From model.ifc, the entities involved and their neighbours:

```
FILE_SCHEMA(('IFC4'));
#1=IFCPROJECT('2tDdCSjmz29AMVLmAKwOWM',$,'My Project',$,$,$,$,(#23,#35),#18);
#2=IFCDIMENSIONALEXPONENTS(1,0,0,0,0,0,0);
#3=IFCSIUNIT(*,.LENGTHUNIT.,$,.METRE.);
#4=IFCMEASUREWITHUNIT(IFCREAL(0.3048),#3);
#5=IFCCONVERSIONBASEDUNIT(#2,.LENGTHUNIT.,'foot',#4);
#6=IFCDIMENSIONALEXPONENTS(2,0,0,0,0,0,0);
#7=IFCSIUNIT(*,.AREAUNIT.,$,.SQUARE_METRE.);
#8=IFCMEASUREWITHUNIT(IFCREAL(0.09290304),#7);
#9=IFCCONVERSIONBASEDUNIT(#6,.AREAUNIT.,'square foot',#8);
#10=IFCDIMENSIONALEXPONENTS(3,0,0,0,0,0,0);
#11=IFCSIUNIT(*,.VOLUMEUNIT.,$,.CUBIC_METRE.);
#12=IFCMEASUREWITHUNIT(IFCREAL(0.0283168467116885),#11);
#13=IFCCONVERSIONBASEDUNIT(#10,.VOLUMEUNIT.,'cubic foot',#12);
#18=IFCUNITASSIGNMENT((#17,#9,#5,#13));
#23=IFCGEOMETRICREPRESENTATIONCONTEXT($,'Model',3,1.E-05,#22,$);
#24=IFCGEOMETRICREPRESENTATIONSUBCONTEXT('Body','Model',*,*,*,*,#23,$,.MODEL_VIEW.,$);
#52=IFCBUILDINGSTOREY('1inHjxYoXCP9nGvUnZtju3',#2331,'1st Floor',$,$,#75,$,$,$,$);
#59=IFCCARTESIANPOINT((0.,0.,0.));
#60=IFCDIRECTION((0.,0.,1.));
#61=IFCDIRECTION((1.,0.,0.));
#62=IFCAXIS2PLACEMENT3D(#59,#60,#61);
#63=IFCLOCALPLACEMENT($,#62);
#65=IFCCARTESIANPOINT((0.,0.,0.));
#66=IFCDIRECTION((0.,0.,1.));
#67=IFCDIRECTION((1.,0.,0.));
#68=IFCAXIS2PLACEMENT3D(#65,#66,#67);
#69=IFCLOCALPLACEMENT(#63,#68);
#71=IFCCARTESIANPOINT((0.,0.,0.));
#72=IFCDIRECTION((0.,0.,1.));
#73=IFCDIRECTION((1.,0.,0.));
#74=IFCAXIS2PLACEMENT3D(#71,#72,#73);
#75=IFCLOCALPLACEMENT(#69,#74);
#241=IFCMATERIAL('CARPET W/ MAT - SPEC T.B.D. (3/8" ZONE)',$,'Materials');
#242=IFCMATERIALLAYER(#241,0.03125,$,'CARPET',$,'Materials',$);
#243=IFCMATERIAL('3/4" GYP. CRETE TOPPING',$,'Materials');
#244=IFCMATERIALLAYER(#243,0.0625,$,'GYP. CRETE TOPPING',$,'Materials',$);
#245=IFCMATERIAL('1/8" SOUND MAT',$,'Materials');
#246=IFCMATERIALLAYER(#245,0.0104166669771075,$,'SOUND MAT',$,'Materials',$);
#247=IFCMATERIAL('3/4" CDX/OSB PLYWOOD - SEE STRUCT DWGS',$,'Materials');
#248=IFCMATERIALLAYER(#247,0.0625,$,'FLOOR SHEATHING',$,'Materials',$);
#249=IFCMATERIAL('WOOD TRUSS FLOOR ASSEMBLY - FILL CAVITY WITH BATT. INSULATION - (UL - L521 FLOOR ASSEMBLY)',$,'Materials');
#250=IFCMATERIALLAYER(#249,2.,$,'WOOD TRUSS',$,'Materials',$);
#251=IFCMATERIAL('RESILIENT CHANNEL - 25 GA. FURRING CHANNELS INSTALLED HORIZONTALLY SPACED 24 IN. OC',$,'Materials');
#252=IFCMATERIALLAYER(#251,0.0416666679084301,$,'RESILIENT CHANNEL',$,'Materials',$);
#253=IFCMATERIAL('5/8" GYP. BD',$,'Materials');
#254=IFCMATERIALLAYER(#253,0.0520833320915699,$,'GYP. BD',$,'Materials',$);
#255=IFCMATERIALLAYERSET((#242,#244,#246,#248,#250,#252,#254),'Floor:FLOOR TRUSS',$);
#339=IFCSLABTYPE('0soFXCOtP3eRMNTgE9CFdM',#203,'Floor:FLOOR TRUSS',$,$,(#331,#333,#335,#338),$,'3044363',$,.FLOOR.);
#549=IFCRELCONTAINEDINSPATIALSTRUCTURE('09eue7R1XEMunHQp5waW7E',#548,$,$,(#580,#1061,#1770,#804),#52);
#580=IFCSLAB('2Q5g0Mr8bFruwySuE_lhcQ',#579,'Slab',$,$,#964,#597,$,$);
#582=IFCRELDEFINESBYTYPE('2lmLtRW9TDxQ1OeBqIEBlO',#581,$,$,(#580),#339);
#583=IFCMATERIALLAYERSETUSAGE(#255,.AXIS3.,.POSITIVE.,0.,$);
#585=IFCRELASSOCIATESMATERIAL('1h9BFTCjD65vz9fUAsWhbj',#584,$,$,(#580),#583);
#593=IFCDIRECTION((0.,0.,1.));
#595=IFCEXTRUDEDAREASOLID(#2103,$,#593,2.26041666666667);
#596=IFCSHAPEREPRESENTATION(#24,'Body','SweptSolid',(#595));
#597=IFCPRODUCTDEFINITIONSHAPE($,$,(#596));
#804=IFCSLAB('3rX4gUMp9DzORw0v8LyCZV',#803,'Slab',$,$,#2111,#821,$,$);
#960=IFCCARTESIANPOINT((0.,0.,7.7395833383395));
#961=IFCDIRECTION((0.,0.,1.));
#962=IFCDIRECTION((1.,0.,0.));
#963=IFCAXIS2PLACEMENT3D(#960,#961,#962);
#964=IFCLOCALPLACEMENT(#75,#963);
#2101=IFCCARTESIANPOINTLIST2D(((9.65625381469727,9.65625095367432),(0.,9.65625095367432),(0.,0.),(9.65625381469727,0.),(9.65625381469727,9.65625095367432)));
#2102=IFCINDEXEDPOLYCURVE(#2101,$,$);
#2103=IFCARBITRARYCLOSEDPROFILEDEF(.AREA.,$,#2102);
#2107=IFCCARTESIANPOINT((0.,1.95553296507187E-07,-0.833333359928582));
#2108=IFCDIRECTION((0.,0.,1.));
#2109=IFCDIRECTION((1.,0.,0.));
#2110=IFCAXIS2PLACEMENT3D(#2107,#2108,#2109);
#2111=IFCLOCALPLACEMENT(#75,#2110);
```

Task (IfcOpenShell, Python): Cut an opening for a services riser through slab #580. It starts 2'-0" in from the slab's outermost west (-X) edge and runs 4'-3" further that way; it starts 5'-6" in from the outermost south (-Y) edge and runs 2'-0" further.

```python
import numpy as np
import ifcopenshell
import ifcopenshell.api.feature
import ifcopenshell.api.geometry
import ifcopenshell.api.root
import ifcopenshell.geom
import ifcopenshell.util.placement
import ifcopenshell.util.representation
import ifcopenshell.util.shape
import ifcopenshell.util.unit

model = ifcopenshell.open("model.ifc")
unit_scale = ifcopenshell.util.unit.calculate_unit_scale(model)
settings = ifcopenshell.geom.settings()


def volume(element):
    """Net volume in cubic metres, openings subtracted."""
    shape = ifcopenshell.geom.create_shape(settings, element)
    return ifcopenshell.util.shape.get_volume(shape.geometry)


slab = model.by_id(580)
before = volume(slab)

# Extent in the slab's own axes, in metres. The edges named are its -X and -Y sides.
slab_shape = ifcopenshell.geom.create_shape(settings, slab)
vertices = ifcopenshell.util.shape.get_vertices(slab_shape.geometry)
x_min, y_min, bottom = vertices.min(axis=0)
top = vertices[:, 2].max()

opening = ifcopenshell.api.root.create_entity(model, ifc_class="IfcOpeningElement", name="Services riser opening", predefined_type="OPENING")
context = ifcopenshell.util.representation.get_context(model, "Model", "Body", "MODEL_VIEW")
width, depth = 1.2954, 0.6096
outline = [(0.0, 0.0), (width, 0.0), (width, depth), (0.0, depth), (0.0, 0.0)]
# Overshoot both faces by 50 mm so the cut is clean.
shape = ifcopenshell.api.geometry.add_slab_representation(
    model, context=context, depth=top - bottom + 0.1, polyline=outline
)
ifcopenshell.api.geometry.assign_representation(model, product=opening, representation=shape)

matrix = ifcopenshell.util.placement.get_local_placement(slab.ObjectPlacement)
matrix[:, 3] = matrix @ np.append(np.array([x_min + 0.6096, y_min + 1.6764, bottom - 0.05]) / unit_scale, 1.0)
ifcopenshell.api.geometry.edit_object_placement(model, product=opening, matrix=matrix, is_si=False)
ifcopenshell.api.feature.add_feature(model, feature=opening, element=slab)

after = volume(slab)

print(f"slab volume {before:.3f} -> {after:.3f} m3")

model.write("model-out.ifc")
```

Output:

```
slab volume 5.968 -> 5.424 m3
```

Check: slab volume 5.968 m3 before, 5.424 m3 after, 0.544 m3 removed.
